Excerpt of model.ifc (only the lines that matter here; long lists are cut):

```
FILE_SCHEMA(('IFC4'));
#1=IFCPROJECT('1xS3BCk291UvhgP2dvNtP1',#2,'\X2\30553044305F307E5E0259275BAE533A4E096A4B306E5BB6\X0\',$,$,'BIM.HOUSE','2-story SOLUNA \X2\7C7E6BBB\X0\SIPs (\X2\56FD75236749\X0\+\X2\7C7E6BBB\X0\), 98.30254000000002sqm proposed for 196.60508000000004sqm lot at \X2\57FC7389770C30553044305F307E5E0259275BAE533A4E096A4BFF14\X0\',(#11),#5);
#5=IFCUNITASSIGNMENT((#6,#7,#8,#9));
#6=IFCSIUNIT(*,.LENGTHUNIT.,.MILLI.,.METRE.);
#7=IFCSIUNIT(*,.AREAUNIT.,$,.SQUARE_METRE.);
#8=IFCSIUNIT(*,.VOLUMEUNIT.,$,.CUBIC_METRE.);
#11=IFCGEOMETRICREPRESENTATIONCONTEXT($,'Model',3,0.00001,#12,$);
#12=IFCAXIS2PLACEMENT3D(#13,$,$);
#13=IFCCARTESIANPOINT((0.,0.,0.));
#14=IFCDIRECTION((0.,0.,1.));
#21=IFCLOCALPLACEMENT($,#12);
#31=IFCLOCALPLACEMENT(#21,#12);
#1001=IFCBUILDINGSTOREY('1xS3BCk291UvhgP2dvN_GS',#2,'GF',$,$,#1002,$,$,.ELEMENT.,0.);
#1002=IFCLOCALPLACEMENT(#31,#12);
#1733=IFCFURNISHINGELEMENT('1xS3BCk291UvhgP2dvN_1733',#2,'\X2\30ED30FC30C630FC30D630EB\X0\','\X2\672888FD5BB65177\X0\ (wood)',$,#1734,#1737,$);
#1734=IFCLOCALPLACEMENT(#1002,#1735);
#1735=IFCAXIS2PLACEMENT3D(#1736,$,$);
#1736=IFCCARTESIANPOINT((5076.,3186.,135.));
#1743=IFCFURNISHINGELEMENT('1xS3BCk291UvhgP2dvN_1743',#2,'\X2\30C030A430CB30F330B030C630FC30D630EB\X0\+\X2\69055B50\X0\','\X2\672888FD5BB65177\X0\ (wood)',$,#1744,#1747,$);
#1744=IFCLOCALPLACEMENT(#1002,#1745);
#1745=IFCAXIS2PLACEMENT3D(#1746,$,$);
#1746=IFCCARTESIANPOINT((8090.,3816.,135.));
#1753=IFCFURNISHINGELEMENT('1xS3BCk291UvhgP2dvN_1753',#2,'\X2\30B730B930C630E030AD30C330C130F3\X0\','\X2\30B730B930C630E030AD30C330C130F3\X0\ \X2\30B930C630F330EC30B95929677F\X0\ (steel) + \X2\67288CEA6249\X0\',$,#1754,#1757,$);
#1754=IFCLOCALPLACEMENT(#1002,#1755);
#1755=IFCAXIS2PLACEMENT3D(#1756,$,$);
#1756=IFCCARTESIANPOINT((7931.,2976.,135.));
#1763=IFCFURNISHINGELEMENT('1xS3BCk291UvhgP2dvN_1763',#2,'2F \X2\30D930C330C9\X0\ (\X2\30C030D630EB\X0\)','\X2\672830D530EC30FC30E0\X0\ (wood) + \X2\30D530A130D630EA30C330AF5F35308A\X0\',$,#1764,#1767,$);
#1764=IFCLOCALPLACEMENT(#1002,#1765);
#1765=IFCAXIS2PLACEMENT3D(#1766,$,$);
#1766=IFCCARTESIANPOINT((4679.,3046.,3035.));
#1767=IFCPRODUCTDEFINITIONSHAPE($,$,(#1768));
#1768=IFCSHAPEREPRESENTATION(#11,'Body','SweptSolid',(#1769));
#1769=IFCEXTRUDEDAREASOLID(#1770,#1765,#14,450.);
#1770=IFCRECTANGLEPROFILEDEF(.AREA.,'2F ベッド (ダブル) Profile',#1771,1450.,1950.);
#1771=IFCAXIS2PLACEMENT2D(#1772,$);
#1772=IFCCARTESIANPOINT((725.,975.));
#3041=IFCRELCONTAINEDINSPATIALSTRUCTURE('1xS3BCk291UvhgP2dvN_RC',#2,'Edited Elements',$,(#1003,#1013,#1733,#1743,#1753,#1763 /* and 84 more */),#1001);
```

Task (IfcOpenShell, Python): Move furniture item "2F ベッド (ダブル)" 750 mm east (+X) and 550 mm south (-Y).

```python
import ifcopenshell
import ifcopenshell.api.geometry
import ifcopenshell.util.placement

model = ifcopenshell.open("model.ifc")

item = model.by_guid("1xS3BCk291UvhgP2dvN_1763")
matrix = ifcopenshell.util.placement.get_local_placement(item.ObjectPlacement)
matrix[0, 3] += 750.0
matrix[1, 3] -= 550.0
ifcopenshell.api.geometry.edit_object_placement(model, product=item, matrix=matrix, is_si=False)

print(ifcopenshell.util.placement.get_local_placement(item.ObjectPlacement).round(3) + 0.0)

model.write("model_edited.ifc")
```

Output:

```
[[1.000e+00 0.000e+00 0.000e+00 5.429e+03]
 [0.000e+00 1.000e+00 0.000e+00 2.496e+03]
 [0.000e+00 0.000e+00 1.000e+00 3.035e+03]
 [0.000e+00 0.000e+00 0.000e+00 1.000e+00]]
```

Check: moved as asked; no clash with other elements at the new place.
